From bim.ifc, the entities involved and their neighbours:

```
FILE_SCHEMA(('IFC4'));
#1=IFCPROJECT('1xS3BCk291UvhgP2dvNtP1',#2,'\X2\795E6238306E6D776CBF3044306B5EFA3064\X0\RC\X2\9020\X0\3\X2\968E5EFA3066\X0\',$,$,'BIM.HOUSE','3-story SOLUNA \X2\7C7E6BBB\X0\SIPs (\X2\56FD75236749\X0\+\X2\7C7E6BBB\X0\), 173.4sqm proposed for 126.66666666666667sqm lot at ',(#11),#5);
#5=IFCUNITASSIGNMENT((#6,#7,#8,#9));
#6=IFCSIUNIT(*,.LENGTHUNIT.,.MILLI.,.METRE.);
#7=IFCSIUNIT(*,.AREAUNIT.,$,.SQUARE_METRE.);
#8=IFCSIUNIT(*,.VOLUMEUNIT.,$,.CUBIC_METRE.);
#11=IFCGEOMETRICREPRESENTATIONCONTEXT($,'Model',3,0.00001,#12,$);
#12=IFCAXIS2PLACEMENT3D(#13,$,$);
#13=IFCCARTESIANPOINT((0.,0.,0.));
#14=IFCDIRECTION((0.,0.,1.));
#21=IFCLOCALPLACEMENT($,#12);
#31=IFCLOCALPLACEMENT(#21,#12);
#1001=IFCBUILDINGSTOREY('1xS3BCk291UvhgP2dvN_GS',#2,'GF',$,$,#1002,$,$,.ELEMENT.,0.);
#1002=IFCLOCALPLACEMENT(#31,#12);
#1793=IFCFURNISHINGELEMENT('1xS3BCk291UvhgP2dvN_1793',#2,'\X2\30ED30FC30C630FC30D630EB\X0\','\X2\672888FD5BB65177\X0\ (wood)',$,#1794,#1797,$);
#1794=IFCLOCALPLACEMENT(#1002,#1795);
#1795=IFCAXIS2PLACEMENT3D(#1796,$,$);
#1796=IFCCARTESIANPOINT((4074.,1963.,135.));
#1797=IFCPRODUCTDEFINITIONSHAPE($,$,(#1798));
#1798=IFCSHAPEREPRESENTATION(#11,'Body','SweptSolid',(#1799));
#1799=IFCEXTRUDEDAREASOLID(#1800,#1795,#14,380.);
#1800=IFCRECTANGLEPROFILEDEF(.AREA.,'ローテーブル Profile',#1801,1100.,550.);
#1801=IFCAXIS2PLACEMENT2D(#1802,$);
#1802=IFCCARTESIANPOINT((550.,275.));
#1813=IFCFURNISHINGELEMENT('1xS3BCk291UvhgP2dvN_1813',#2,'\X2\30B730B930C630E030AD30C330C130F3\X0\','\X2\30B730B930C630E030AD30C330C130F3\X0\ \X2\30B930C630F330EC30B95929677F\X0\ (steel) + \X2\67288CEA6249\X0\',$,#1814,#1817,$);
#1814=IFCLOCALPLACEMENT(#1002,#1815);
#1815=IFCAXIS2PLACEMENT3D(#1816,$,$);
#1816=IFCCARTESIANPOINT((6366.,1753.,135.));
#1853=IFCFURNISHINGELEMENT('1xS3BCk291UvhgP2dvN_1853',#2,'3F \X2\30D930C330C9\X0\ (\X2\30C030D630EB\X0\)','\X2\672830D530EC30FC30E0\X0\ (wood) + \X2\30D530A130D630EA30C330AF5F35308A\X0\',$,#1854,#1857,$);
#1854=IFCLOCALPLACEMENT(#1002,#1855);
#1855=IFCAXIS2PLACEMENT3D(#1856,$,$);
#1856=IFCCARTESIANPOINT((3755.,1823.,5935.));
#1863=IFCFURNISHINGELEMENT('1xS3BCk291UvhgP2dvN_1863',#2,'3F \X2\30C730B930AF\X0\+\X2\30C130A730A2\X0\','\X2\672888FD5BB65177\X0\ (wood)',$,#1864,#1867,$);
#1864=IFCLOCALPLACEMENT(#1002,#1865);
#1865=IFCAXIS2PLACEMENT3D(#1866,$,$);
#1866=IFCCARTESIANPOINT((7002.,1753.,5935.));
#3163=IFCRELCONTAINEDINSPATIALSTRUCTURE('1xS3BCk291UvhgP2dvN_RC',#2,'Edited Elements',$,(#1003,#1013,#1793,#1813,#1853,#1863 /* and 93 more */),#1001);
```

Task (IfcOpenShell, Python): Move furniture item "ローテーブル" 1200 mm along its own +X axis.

```python
import ifcopenshell
import ifcopenshell.api.geometry
import ifcopenshell.util.placement
import ifcopenshell.util.unit

model = ifcopenshell.open("bim.ifc")
unit_scale = ifcopenshell.util.unit.calculate_unit_scale(model)

item = model.by_id(1793)
matrix = ifcopenshell.util.placement.get_local_placement(item.ObjectPlacement)
matrix[:3, 3] += matrix[:3, 0] * 1.2 / unit_scale
ifcopenshell.api.geometry.edit_object_placement(model, product=item, matrix=matrix, is_si=False)

print(ifcopenshell.util.placement.get_local_placement(item.ObjectPlacement).round(3) + 0.0)

model.write("bim-out.ifc")
```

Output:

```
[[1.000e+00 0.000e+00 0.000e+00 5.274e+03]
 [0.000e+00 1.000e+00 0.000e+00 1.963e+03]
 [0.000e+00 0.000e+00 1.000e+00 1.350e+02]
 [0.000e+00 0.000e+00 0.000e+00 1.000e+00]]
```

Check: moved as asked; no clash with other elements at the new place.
